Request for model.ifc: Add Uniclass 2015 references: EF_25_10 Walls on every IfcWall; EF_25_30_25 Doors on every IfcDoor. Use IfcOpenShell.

First a look at what the model holds.

```python
import ifcopenshell

model = ifcopenshell.open("model.ifc")
print(model.schema)
print("classifications:", [c.Name for c in model.by_type("IfcClassification")])
for ifc_class in ("IfcDoor", "IfcRoof", "IfcStair", "IfcWall", "IfcWindow"):
    print(ifc_class, len(model.by_type(ifc_class)))
```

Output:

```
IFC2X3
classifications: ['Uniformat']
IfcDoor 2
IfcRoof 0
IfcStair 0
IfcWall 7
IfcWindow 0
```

```python
import ifcopenshell
import ifcopenshell.api.classification

model = ifcopenshell.open("model.ifc")

# IFC2X3 requires Source and Edition and has no link from the project to the system.
system = model.create_entity("IfcClassification", Source="NBS", Edition="2015", Name="Uniclass 2015")

codes = {
    "IfcWall": ("EF_25_10", "Walls"),
    "IfcDoor": ("EF_25_30_25", "Doors"),
}
for ifc_class, (code, name) in codes.items():
    products = model.by_type(ifc_class)
    ifcopenshell.api.classification.add_reference(
        model, products=products, classification=system, identification=code, name=name
    )
    print(code, len(products))

model.write("model_v2.ifc")
```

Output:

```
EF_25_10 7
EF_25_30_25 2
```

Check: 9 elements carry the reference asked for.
